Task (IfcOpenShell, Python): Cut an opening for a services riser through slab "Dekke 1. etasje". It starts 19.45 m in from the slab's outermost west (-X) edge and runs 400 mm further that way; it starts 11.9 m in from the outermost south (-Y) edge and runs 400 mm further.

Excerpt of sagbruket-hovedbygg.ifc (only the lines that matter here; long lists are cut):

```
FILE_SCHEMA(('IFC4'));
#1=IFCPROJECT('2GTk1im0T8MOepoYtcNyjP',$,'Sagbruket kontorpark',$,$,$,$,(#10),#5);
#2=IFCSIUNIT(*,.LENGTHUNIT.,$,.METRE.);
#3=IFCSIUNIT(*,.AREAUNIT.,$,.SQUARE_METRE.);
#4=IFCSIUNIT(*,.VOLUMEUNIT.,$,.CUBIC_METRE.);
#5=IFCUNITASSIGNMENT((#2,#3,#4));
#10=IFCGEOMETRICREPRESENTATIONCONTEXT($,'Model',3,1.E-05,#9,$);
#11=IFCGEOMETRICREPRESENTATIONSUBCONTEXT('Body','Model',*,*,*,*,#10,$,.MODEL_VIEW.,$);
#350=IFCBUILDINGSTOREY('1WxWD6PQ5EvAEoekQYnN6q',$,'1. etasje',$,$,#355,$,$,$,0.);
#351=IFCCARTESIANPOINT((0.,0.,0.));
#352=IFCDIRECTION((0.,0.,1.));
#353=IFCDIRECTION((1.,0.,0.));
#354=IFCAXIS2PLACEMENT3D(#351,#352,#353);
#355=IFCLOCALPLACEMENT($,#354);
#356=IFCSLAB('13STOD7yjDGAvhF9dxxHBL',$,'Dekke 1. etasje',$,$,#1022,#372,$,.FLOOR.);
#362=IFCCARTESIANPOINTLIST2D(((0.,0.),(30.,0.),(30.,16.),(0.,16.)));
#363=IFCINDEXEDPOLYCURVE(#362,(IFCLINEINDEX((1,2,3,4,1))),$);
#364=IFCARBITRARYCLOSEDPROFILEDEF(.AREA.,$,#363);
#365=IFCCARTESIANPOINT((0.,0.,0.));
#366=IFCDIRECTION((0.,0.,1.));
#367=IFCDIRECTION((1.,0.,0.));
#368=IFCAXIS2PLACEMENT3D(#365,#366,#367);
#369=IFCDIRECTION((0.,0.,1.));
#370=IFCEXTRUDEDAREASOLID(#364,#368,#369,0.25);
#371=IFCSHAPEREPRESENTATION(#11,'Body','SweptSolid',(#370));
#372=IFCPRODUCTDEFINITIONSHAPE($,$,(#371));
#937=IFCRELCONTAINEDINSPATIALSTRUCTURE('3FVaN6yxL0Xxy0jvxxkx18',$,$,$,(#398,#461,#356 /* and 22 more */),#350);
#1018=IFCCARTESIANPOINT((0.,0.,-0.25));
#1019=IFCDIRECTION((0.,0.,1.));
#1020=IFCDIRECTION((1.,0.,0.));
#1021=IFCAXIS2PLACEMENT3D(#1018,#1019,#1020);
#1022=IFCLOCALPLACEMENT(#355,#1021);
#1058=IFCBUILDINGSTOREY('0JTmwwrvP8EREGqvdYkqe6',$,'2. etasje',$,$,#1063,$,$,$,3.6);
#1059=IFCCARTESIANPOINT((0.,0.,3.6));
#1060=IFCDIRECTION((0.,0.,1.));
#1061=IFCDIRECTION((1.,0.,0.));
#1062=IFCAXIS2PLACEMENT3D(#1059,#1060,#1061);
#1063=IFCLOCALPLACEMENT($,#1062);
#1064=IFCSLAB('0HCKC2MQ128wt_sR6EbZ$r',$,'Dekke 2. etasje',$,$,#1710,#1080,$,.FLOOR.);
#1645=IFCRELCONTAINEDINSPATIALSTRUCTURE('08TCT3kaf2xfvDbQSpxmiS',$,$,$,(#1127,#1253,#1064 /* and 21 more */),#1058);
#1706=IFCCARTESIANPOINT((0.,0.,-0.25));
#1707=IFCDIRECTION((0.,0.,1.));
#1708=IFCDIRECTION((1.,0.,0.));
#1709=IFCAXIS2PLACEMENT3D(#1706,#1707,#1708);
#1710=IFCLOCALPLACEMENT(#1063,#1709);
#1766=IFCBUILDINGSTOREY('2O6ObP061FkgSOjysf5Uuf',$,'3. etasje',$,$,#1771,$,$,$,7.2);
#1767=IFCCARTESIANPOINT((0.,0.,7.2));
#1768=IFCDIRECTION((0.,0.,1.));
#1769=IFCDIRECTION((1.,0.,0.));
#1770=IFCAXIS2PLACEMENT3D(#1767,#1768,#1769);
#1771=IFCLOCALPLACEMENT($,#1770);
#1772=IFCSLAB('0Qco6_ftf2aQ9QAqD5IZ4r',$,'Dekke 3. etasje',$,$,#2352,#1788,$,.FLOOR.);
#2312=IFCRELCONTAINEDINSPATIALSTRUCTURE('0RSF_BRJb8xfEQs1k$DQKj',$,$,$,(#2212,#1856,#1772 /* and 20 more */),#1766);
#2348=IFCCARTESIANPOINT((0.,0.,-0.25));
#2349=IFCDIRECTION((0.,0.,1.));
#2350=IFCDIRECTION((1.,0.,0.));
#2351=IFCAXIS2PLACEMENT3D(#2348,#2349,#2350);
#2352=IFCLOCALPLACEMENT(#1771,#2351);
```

```python
import numpy as np
import ifcopenshell
import ifcopenshell.api.feature
import ifcopenshell.api.geometry
import ifcopenshell.api.root
import ifcopenshell.geom
import ifcopenshell.util.placement
import ifcopenshell.util.representation
import ifcopenshell.util.shape
import ifcopenshell.util.unit

model = ifcopenshell.open("sagbruket-hovedbygg.ifc")
unit_scale = ifcopenshell.util.unit.calculate_unit_scale(model)
settings = ifcopenshell.geom.settings()


def volume(element):
    """Net volume in cubic metres, openings subtracted."""
    shape = ifcopenshell.geom.create_shape(settings, element)
    return ifcopenshell.util.shape.get_volume(shape.geometry)


slab = model.by_guid("13STOD7yjDGAvhF9dxxHBL")
before = volume(slab)

# Extent in the slab's own axes, in metres. The edges named are its -X and -Y sides.
slab_shape = ifcopenshell.geom.create_shape(settings, slab)
vertices = ifcopenshell.util.shape.get_vertices(slab_shape.geometry)
x_min, y_min, bottom = vertices.min(axis=0)
top = vertices[:, 2].max()

opening = ifcopenshell.api.root.create_entity(model, ifc_class="IfcOpeningElement", name="Services riser opening", predefined_type="OPENING")
context = ifcopenshell.util.representation.get_context(model, "Model", "Body", "MODEL_VIEW")
width, depth = 0.4, 0.4
outline = [(0.0, 0.0), (width, 0.0), (width, depth), (0.0, depth), (0.0, 0.0)]
# Overshoot both faces by 50 mm so the cut is clean.
shape = ifcopenshell.api.geometry.add_slab_representation(
    model, context=context, depth=top - bottom + 0.1, polyline=outline
)
ifcopenshell.api.geometry.assign_representation(model, product=opening, representation=shape)

matrix = ifcopenshell.util.placement.get_local_placement(slab.ObjectPlacement)
matrix[:, 3] = matrix @ np.append(np.array([x_min + 19.45, y_min + 11.9, bottom - 0.05]) / unit_scale, 1.0)
ifcopenshell.api.geometry.edit_object_placement(model, product=opening, matrix=matrix, is_si=False)
ifcopenshell.api.feature.add_feature(model, feature=opening, element=slab)

after = volume(slab)

print(f"slab volume {before:.3f} -> {after:.3f} m3")

model.write("sagbruket-hovedbygg_rev.ifc")
```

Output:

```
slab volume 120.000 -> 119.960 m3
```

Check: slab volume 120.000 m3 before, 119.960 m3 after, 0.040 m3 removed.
